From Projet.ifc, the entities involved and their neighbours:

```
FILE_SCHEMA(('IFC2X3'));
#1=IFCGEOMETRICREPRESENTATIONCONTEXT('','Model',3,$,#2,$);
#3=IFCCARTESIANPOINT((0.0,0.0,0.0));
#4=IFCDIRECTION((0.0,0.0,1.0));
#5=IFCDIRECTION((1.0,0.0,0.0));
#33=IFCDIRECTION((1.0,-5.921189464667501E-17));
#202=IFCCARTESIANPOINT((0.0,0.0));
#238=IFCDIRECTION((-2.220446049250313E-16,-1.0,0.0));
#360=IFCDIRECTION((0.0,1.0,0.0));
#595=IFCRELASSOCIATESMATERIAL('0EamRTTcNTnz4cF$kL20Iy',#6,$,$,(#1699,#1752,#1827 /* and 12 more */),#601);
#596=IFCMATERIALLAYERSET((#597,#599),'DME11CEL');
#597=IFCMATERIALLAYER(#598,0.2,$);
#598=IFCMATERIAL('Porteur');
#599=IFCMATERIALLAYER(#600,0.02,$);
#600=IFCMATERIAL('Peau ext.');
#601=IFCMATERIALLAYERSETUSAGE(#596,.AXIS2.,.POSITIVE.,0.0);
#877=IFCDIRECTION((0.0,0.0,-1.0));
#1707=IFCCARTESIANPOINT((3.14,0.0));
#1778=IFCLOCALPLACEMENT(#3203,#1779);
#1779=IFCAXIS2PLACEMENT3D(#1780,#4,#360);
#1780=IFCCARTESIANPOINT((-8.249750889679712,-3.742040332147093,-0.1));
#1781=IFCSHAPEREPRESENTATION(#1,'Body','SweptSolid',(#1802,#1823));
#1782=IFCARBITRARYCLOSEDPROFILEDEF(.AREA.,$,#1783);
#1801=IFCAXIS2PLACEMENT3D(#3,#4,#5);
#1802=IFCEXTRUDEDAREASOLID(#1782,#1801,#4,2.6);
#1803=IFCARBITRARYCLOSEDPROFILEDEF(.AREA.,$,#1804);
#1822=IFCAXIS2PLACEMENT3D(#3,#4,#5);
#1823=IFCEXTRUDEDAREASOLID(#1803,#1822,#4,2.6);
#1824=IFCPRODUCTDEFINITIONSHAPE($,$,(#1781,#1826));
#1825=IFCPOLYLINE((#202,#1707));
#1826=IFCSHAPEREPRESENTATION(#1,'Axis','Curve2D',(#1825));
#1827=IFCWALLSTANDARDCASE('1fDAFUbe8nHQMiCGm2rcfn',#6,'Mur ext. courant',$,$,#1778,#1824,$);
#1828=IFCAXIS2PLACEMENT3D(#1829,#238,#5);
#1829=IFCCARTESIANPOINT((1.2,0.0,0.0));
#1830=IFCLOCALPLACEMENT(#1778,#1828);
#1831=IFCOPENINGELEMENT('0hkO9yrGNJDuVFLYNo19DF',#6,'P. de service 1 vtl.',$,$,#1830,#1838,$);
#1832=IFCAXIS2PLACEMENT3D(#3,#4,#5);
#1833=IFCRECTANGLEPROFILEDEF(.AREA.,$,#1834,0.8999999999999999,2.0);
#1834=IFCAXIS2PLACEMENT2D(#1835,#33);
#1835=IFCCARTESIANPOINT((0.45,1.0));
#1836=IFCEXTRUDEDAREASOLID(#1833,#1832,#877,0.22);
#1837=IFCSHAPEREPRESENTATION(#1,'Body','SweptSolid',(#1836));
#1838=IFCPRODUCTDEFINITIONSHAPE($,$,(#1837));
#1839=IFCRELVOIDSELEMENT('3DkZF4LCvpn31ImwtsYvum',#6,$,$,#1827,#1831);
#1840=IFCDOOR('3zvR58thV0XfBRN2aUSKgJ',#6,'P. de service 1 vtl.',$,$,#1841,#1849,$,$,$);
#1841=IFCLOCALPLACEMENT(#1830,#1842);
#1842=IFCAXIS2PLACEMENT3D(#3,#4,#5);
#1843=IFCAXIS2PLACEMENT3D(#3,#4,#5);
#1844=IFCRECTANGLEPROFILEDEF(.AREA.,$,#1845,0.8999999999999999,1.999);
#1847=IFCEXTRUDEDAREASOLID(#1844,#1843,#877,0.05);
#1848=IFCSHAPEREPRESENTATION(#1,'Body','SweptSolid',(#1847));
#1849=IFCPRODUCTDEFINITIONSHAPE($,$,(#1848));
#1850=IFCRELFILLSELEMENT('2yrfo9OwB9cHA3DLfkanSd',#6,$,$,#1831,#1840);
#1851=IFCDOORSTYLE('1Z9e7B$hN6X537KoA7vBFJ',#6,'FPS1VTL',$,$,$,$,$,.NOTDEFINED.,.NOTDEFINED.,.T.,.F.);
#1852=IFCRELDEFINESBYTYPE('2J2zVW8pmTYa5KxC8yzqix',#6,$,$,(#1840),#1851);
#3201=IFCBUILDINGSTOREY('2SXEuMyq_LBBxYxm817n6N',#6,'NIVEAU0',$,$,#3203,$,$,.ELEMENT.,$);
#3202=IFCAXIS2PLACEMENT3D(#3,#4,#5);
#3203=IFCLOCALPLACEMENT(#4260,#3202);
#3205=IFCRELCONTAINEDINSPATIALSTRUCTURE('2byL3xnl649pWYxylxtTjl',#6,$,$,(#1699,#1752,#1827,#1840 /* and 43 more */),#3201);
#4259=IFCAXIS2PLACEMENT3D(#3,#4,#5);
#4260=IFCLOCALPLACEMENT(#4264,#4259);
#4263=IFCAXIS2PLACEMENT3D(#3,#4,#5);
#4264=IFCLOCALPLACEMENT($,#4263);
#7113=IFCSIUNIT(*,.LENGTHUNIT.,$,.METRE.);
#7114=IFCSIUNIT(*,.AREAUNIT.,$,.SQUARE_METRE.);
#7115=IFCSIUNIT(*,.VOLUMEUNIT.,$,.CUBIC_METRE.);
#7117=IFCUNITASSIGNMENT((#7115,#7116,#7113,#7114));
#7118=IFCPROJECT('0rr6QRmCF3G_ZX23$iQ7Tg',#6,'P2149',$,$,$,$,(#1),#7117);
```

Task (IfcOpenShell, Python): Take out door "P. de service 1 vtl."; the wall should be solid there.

```python
import ifcopenshell
import ifcopenshell.api.feature
import ifcopenshell.api.root
import ifcopenshell.geom
import ifcopenshell.util.shape

model = ifcopenshell.open("Projet.ifc")
settings = ifcopenshell.geom.settings()


def volume(element):
    """Net volume in cubic metres, openings subtracted."""
    shape = ifcopenshell.geom.create_shape(settings, element)
    return ifcopenshell.util.shape.get_volume(shape.geometry)


door = model.by_guid("3zvR58thV0XfBRN2aUSKgJ")
opening = door.FillsVoids[0].RelatingOpeningElement
wall = opening.VoidsElements[0].RelatingBuildingElement
before = volume(wall)

ifcopenshell.api.root.remove_product(model, product=door)
ifcopenshell.api.feature.remove_feature(model, feature=opening)

after = volume(wall)

print(f"wall volume {before:.3f} -> {after:.3f} m3")

model.write("Projet-out.ifc")
```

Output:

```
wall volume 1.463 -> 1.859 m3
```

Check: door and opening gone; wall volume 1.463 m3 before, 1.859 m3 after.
